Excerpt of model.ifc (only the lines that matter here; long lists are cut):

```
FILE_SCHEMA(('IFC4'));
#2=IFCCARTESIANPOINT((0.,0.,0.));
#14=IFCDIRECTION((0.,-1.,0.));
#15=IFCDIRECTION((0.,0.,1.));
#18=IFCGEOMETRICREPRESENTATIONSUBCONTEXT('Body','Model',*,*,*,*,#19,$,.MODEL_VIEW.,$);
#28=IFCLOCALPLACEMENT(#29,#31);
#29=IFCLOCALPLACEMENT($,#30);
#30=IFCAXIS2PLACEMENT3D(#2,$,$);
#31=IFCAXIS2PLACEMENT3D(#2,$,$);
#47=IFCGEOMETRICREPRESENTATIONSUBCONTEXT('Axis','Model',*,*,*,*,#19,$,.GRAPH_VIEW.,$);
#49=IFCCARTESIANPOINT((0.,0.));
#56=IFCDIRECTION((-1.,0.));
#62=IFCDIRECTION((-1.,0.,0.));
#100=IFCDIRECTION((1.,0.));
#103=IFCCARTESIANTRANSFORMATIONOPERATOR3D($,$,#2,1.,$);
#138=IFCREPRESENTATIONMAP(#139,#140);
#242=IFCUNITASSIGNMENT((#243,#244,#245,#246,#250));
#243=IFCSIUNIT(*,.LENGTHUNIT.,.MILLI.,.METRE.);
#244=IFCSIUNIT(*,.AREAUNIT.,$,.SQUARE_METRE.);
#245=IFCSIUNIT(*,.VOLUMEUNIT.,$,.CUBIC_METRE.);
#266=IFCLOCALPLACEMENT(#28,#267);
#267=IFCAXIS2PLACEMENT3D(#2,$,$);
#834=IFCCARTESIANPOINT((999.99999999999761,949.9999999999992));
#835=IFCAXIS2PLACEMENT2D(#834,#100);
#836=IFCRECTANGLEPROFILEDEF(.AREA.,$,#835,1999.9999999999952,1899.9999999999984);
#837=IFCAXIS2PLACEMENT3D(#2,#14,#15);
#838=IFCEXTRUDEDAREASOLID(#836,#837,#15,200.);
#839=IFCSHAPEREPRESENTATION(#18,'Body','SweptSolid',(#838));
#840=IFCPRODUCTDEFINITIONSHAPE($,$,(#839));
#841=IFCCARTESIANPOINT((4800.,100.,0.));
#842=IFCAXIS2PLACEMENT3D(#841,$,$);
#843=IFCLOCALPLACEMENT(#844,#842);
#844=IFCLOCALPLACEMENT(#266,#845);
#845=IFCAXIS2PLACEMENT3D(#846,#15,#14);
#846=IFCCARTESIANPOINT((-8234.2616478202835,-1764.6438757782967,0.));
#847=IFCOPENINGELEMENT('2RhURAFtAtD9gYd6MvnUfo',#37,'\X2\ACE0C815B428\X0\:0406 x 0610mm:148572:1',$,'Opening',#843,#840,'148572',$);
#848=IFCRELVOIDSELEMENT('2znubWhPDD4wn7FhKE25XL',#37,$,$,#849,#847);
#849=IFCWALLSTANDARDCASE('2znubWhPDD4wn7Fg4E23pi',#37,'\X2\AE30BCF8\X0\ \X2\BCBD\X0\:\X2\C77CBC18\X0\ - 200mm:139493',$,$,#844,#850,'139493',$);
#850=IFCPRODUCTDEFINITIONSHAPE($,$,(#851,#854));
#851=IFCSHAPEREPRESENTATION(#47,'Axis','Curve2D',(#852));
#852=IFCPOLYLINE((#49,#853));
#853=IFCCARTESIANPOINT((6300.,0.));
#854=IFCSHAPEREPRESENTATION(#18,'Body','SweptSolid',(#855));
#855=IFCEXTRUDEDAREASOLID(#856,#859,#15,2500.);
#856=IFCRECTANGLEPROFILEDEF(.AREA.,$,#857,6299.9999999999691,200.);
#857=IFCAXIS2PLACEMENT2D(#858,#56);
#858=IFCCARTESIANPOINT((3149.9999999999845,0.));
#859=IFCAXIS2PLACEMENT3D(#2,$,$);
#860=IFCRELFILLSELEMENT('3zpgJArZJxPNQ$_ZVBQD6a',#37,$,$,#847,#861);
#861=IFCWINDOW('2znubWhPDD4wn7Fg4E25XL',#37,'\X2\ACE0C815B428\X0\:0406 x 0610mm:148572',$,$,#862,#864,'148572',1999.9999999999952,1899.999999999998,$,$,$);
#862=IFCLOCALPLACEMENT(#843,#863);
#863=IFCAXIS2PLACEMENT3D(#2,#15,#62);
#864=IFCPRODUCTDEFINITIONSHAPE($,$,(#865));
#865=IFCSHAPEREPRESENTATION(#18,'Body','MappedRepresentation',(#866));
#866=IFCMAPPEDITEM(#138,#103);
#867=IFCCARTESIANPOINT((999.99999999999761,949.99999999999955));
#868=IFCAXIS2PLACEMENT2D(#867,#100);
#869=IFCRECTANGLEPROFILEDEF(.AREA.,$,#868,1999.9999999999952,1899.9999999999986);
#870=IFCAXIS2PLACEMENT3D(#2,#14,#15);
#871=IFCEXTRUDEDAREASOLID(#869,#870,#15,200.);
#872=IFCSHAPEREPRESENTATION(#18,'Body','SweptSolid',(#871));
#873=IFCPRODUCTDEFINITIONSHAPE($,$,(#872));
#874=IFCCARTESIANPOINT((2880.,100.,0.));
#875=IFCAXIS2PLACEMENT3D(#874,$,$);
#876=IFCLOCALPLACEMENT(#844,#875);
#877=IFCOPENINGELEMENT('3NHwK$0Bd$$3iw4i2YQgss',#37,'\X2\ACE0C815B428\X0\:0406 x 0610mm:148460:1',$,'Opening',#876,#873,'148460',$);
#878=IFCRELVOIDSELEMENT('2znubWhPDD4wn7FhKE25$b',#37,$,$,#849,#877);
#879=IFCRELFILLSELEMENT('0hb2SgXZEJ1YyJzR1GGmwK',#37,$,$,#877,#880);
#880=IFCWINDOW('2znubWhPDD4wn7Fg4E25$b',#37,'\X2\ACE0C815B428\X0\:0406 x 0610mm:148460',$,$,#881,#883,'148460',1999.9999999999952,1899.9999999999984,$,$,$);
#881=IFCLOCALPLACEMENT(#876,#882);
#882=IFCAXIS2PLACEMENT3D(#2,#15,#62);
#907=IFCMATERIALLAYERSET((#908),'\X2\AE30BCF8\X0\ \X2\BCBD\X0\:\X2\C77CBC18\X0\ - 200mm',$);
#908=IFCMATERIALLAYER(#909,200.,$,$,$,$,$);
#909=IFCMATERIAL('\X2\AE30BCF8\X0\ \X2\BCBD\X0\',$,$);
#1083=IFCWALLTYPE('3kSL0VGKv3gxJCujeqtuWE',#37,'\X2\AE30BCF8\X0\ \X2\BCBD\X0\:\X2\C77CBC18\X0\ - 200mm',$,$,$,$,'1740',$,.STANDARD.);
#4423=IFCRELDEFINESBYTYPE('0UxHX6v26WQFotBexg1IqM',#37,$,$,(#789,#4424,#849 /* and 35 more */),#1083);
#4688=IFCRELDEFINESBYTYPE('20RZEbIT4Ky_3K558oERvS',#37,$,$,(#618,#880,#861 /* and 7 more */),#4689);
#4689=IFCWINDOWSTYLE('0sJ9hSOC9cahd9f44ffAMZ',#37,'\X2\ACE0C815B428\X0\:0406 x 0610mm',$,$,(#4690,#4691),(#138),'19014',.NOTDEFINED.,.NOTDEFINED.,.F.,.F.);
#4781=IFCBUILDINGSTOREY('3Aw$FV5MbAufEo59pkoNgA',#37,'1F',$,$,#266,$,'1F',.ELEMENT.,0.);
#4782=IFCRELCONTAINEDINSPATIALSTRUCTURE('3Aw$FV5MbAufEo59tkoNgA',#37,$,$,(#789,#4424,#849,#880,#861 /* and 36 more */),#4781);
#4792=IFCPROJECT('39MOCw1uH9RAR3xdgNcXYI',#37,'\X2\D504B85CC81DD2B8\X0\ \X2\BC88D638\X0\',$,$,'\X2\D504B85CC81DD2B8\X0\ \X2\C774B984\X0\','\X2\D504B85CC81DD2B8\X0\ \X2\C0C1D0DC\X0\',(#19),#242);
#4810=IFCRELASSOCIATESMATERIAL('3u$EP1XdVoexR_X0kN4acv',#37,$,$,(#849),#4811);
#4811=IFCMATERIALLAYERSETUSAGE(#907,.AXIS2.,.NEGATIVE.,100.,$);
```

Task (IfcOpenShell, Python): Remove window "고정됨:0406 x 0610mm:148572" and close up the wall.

```python
import ifcopenshell
import ifcopenshell.api.feature
import ifcopenshell.api.root
import ifcopenshell.geom
import ifcopenshell.util.shape

model = ifcopenshell.open("model.ifc")
settings = ifcopenshell.geom.settings()


def volume(element):
    """Net volume in cubic metres, openings subtracted."""
    shape = ifcopenshell.geom.create_shape(settings, element)
    return ifcopenshell.util.shape.get_volume(shape.geometry)


window = model.by_guid("2znubWhPDD4wn7Fg4E25XL")
opening = window.FillsVoids[0].RelatingOpeningElement
wall = opening.VoidsElements[0].RelatingBuildingElement
before = volume(wall)

ifcopenshell.api.root.remove_product(model, product=window)
ifcopenshell.api.feature.remove_feature(model, feature=opening)

after = volume(wall)

print(f"wall volume {before:.3f} -> {after:.3f} m3")

model.write("model_edited.ifc")
```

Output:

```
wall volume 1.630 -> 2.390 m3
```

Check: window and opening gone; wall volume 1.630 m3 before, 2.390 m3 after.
